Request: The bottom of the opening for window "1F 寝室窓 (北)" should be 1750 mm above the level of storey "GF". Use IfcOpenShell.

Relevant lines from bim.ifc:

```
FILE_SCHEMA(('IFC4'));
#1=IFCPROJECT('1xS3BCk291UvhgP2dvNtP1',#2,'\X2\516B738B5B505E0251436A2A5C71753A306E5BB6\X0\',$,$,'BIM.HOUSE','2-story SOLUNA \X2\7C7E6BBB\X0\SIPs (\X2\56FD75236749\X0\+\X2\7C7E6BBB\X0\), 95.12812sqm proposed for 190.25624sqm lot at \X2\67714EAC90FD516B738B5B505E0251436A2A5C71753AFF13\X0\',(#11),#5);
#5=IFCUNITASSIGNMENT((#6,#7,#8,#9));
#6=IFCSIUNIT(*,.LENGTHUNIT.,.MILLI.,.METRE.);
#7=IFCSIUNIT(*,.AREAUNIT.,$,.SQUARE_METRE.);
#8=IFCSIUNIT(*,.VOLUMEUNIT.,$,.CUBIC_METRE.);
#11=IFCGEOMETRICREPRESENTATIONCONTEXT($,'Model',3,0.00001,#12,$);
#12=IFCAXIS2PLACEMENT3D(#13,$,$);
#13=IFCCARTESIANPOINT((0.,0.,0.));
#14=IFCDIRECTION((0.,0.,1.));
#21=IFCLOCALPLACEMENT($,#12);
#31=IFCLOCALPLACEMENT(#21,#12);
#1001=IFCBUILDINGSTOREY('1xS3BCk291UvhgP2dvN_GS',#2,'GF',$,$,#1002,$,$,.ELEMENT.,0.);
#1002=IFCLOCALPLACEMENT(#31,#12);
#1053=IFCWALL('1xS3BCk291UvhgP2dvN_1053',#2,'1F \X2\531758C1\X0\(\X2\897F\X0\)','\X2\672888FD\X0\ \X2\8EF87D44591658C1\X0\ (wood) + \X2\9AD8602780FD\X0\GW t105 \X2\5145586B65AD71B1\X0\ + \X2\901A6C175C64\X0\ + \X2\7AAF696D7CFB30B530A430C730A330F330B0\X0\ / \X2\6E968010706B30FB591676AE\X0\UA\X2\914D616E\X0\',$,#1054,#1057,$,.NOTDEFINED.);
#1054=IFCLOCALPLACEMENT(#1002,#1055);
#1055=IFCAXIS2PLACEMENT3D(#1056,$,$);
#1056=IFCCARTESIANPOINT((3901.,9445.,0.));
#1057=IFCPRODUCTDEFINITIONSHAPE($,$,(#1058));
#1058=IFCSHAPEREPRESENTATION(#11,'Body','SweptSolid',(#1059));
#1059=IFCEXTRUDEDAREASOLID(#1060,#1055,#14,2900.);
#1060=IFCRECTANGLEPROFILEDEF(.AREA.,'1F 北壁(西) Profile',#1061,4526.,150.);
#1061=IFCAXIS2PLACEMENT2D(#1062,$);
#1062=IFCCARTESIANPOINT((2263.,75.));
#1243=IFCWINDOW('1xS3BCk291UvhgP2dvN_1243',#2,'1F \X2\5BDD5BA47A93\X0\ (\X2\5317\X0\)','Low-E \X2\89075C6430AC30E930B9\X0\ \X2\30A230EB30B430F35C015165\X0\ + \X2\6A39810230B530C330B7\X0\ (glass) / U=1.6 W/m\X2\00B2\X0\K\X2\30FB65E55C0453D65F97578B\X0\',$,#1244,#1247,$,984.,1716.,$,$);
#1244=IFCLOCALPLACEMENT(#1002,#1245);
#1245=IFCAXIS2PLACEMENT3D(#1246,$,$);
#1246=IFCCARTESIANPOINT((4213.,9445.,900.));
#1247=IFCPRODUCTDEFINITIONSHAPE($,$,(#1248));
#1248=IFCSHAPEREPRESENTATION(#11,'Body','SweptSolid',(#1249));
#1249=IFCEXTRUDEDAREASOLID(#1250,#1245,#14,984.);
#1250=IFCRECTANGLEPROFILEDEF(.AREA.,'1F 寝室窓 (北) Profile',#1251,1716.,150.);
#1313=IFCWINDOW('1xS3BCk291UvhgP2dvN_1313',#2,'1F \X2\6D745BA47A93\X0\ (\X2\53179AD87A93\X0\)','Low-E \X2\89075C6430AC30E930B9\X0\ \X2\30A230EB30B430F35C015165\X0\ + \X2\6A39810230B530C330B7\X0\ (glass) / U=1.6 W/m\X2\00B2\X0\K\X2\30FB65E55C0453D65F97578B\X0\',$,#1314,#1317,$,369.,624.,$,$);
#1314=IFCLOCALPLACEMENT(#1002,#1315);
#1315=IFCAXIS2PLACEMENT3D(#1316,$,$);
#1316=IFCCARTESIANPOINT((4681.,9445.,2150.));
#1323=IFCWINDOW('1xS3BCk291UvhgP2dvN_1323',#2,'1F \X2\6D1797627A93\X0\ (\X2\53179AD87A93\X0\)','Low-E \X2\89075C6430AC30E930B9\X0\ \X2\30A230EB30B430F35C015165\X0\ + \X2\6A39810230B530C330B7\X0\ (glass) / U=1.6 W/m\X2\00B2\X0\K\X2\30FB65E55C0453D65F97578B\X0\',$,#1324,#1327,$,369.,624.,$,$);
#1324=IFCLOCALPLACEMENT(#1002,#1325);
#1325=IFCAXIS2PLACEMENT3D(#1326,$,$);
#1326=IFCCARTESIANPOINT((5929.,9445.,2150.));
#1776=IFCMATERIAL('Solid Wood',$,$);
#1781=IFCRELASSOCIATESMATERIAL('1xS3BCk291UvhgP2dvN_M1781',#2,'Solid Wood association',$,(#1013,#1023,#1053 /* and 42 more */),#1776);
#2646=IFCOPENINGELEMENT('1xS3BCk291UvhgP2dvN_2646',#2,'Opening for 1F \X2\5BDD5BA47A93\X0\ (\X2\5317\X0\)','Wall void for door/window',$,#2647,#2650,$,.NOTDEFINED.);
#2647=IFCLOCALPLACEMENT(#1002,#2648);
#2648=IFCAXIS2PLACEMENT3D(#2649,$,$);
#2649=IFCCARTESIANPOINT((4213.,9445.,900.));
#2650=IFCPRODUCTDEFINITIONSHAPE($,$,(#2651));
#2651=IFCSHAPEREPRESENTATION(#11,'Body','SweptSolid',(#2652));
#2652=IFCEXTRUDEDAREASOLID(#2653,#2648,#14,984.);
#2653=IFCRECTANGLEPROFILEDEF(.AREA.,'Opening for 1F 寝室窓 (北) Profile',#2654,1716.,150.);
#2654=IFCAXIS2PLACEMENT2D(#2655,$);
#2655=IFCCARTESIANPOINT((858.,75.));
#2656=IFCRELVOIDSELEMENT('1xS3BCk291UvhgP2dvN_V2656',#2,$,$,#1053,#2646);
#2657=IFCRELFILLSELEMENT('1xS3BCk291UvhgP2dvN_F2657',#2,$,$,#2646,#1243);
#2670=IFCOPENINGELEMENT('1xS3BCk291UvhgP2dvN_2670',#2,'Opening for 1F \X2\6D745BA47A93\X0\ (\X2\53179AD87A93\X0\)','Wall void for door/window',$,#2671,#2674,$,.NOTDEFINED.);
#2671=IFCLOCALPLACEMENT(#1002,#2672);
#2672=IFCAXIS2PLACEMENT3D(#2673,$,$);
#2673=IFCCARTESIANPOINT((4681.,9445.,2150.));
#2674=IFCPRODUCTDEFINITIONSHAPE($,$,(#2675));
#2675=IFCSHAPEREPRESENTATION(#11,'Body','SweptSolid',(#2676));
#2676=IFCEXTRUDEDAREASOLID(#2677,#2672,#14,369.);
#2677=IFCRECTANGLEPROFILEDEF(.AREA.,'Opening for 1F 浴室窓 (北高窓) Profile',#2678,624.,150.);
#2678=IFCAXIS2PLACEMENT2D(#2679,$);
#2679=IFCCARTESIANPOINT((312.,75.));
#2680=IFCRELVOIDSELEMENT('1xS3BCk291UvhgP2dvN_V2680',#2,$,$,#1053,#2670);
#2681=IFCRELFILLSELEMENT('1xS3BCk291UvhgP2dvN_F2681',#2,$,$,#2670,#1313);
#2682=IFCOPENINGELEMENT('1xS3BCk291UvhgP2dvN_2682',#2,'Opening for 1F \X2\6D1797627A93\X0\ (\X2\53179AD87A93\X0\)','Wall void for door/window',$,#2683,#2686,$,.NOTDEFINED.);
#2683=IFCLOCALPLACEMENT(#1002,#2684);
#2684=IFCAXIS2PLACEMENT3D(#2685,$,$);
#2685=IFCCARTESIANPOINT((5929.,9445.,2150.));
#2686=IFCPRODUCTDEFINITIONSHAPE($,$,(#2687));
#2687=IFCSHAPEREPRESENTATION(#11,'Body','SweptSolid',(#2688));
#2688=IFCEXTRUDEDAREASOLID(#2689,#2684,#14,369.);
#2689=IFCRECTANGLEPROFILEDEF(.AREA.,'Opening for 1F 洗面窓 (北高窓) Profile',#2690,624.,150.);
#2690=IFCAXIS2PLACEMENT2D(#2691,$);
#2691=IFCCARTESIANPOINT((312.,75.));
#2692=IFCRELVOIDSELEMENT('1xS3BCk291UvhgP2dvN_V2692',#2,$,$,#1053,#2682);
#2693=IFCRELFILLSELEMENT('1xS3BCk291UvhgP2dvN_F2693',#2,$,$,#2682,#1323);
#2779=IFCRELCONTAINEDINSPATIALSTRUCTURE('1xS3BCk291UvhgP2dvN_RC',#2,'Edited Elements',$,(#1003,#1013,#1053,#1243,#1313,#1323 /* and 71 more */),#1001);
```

```python
import numpy as np
import ifcopenshell
import ifcopenshell.api.geometry
import ifcopenshell.geom
import ifcopenshell.util.element
import ifcopenshell.util.placement
import ifcopenshell.util.shape
import ifcopenshell.util.unit

model = ifcopenshell.open("bim.ifc")
unit_scale = ifcopenshell.util.unit.calculate_unit_scale(model)

window = model.by_id(1243)
opening = window.FillsVoids[0].RelatingOpeningElement
storey = ifcopenshell.util.element.get_container(window, ifc_class="IfcBuildingStorey")
level = ifcopenshell.util.placement.get_local_placement(storey.ObjectPlacement)[2, 3]

# The opening's origin need not be at the sill, so measure its lowest point.
shape = ifcopenshell.geom.create_shape(ifcopenshell.geom.settings(), opening)
bottom = ifcopenshell.util.shape.get_shape_bottom_elevation(shape, shape.geometry) / unit_scale
dz = level + 1.75 / unit_scale - bottom

shift = np.array([0.0, 0.0, dz])
# The window is not placed relative to its opening, so move both.
for product in (opening, window):
    matrix = ifcopenshell.util.placement.get_local_placement(product.ObjectPlacement)
    matrix[:3, 3] += shift
    ifcopenshell.api.geometry.edit_object_placement(model, product=product, matrix=matrix, is_si=False)

print(f"moved by {dz * unit_scale:+.3f} m")

model.write("bim_edited.ifc")
```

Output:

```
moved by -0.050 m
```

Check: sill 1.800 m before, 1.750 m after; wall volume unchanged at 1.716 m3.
